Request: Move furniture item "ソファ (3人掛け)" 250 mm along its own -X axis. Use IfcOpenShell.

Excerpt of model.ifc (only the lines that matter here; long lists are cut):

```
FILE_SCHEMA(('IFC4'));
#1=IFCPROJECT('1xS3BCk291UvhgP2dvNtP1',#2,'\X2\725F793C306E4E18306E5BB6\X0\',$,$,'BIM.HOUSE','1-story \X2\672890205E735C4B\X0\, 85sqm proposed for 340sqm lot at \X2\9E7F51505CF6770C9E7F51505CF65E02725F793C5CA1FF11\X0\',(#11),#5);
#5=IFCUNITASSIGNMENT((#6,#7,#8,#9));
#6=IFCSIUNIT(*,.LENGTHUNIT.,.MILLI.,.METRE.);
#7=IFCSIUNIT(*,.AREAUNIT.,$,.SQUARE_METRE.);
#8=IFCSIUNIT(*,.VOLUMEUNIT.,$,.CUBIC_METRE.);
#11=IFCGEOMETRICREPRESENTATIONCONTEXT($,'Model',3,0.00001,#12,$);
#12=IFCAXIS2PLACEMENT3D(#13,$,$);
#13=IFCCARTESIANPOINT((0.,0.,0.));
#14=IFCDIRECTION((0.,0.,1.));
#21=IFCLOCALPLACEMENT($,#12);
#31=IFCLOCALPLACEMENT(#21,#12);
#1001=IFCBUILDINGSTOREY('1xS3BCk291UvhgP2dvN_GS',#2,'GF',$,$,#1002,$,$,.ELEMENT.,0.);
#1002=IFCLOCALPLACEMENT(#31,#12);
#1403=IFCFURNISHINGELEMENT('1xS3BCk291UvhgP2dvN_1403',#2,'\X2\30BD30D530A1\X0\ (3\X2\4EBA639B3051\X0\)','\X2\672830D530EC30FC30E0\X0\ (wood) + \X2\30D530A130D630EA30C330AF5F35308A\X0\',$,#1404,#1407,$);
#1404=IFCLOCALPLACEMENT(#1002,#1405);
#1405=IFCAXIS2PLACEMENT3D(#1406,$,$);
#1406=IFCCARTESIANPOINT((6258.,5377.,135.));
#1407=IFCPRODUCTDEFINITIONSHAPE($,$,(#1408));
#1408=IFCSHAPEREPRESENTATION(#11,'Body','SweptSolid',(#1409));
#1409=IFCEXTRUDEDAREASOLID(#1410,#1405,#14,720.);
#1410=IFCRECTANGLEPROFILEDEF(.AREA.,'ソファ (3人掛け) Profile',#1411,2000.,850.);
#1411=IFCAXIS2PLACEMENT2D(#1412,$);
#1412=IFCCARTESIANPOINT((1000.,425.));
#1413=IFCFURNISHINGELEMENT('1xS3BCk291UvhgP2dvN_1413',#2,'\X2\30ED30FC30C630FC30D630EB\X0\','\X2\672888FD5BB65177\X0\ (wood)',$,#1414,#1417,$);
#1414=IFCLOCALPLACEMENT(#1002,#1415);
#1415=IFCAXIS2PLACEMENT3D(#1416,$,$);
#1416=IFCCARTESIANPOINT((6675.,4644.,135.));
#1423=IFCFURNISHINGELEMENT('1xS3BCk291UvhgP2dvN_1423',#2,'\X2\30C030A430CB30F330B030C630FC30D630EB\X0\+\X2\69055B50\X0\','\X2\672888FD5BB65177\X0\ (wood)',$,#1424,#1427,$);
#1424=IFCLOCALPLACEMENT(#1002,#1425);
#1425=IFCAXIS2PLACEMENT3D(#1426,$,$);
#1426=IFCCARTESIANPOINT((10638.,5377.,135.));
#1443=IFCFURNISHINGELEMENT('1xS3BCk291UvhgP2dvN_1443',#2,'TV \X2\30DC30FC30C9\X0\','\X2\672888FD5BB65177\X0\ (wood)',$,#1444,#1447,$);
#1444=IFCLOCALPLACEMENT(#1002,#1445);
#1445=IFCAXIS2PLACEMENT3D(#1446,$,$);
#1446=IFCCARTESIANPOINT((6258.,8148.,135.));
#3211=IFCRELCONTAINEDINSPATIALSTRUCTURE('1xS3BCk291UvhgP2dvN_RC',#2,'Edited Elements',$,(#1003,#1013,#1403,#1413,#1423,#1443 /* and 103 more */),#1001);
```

```python
import ifcopenshell
import ifcopenshell.api.geometry
import ifcopenshell.util.placement

model = ifcopenshell.open("model.ifc")

item = model.by_id(1403)
matrix = ifcopenshell.util.placement.get_local_placement(item.ObjectPlacement)
matrix[:3, 3] -= matrix[:3, 0] * 250.0
ifcopenshell.api.geometry.edit_object_placement(model, product=item, matrix=matrix, is_si=False)

print(ifcopenshell.util.placement.get_local_placement(item.ObjectPlacement).round(3) + 0.0)

model.write("model-out.ifc")
```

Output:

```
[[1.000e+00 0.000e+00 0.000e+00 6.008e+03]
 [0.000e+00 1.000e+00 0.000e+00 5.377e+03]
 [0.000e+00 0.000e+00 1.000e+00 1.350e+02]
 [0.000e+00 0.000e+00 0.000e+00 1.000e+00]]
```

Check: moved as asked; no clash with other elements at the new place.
